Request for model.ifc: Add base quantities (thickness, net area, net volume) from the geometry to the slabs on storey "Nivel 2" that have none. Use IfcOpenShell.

First a look at what the model holds.

```python
import ifcopenshell
import ifcopenshell.util.element
import ifcopenshell.util.unit

model = ifcopenshell.open("model.ifc")
print(model.schema)
for unit_type in ("LENGTHUNIT", "AREAUNIT", "VOLUMEUNIT"):
    print(unit_type, ifcopenshell.util.unit.calculate_unit_scale(model, unit_type))
storey = next(s for s in model.by_type("IfcBuildingStorey") if s.Name == "Nivel 2")
slabs = [e for e in ifcopenshell.util.element.get_decomposition(storey) if e.is_a("IfcSlab")]
for e in sorted(slabs, key=lambda e: e.id()):
    print(e.id(), e.is_a(), e.Name, list(ifcopenshell.util.element.get_psets(e, qtos_only=True)), sep=" | ")
```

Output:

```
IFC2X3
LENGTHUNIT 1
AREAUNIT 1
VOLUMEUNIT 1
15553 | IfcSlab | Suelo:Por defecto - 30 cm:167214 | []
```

```python
import ifcopenshell
import ifcopenshell.api.pset
import ifcopenshell.geom
import ifcopenshell.util.element
import ifcopenshell.util.shape
import ifcopenshell.util.unit

model = ifcopenshell.open("model.ifc")
unit_scale = ifcopenshell.util.unit.calculate_unit_scale(model)
area_scale = ifcopenshell.util.unit.calculate_unit_scale(model, "AREAUNIT")
volume_scale = ifcopenshell.util.unit.calculate_unit_scale(model, "VOLUMEUNIT")
settings = ifcopenshell.geom.settings()

storey = next(s for s in model.by_type("IfcBuildingStorey") if s.Name == "Nivel 2")
slabs = [e for e in ifcopenshell.util.element.get_decomposition(storey) if e.is_a("IfcSlab")]

for e in sorted(slabs, key=lambda e: e.id()):
    if ifcopenshell.util.element.get_psets(e, qtos_only=True, should_inherit=False):
        continue
    # Geometry comes back in metres, in the element's own axes.
    shape = ifcopenshell.geom.create_shape(settings, e)
    values = {
        "Width": ifcopenshell.util.shape.get_z(shape.geometry) / unit_scale,
        "NetArea": ifcopenshell.util.shape.get_footprint_area(shape.geometry) / area_scale,
        "NetVolume": ifcopenshell.util.shape.get_volume(shape.geometry) / volume_scale,
    }
    qto = ifcopenshell.api.pset.add_qto(model, product=e, name="BaseQuantities")
    ifcopenshell.api.pset.edit_qto(model, qto=qto, properties=values)
    print(e.id(), {k: round(v, 3) for k, v in values.items()})

model.write("model_rev.ifc")
```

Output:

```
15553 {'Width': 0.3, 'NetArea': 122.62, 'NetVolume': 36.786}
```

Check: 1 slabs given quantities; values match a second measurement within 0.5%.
